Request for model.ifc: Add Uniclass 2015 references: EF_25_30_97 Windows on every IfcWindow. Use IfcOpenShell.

First a look at what the model holds.

```python
import ifcopenshell

model = ifcopenshell.open("model.ifc")
print(model.schema)
print("classifications:", [c.Name for c in model.by_type("IfcClassification")])
for ifc_class in ("IfcDoor", "IfcRoof", "IfcStair", "IfcWall", "IfcWindow"):
    print(ifc_class, len(model.by_type(ifc_class)))
```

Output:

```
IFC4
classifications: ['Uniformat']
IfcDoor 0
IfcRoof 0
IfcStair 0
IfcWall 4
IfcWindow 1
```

```python
import ifcopenshell
import ifcopenshell.api.classification

model = ifcopenshell.open("model.ifc")

system = ifcopenshell.api.classification.add_classification(model, classification="Uniclass 2015")

codes = {
    "IfcWindow": ("EF_25_30_97", "Windows"),
}
for ifc_class, (code, name) in codes.items():
    products = model.by_type(ifc_class)
    ifcopenshell.api.classification.add_reference(
        model, products=products, classification=system, identification=code, name=name
    )
    print(code, len(products))

model.write("model_v2.ifc")
```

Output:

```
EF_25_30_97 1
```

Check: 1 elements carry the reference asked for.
